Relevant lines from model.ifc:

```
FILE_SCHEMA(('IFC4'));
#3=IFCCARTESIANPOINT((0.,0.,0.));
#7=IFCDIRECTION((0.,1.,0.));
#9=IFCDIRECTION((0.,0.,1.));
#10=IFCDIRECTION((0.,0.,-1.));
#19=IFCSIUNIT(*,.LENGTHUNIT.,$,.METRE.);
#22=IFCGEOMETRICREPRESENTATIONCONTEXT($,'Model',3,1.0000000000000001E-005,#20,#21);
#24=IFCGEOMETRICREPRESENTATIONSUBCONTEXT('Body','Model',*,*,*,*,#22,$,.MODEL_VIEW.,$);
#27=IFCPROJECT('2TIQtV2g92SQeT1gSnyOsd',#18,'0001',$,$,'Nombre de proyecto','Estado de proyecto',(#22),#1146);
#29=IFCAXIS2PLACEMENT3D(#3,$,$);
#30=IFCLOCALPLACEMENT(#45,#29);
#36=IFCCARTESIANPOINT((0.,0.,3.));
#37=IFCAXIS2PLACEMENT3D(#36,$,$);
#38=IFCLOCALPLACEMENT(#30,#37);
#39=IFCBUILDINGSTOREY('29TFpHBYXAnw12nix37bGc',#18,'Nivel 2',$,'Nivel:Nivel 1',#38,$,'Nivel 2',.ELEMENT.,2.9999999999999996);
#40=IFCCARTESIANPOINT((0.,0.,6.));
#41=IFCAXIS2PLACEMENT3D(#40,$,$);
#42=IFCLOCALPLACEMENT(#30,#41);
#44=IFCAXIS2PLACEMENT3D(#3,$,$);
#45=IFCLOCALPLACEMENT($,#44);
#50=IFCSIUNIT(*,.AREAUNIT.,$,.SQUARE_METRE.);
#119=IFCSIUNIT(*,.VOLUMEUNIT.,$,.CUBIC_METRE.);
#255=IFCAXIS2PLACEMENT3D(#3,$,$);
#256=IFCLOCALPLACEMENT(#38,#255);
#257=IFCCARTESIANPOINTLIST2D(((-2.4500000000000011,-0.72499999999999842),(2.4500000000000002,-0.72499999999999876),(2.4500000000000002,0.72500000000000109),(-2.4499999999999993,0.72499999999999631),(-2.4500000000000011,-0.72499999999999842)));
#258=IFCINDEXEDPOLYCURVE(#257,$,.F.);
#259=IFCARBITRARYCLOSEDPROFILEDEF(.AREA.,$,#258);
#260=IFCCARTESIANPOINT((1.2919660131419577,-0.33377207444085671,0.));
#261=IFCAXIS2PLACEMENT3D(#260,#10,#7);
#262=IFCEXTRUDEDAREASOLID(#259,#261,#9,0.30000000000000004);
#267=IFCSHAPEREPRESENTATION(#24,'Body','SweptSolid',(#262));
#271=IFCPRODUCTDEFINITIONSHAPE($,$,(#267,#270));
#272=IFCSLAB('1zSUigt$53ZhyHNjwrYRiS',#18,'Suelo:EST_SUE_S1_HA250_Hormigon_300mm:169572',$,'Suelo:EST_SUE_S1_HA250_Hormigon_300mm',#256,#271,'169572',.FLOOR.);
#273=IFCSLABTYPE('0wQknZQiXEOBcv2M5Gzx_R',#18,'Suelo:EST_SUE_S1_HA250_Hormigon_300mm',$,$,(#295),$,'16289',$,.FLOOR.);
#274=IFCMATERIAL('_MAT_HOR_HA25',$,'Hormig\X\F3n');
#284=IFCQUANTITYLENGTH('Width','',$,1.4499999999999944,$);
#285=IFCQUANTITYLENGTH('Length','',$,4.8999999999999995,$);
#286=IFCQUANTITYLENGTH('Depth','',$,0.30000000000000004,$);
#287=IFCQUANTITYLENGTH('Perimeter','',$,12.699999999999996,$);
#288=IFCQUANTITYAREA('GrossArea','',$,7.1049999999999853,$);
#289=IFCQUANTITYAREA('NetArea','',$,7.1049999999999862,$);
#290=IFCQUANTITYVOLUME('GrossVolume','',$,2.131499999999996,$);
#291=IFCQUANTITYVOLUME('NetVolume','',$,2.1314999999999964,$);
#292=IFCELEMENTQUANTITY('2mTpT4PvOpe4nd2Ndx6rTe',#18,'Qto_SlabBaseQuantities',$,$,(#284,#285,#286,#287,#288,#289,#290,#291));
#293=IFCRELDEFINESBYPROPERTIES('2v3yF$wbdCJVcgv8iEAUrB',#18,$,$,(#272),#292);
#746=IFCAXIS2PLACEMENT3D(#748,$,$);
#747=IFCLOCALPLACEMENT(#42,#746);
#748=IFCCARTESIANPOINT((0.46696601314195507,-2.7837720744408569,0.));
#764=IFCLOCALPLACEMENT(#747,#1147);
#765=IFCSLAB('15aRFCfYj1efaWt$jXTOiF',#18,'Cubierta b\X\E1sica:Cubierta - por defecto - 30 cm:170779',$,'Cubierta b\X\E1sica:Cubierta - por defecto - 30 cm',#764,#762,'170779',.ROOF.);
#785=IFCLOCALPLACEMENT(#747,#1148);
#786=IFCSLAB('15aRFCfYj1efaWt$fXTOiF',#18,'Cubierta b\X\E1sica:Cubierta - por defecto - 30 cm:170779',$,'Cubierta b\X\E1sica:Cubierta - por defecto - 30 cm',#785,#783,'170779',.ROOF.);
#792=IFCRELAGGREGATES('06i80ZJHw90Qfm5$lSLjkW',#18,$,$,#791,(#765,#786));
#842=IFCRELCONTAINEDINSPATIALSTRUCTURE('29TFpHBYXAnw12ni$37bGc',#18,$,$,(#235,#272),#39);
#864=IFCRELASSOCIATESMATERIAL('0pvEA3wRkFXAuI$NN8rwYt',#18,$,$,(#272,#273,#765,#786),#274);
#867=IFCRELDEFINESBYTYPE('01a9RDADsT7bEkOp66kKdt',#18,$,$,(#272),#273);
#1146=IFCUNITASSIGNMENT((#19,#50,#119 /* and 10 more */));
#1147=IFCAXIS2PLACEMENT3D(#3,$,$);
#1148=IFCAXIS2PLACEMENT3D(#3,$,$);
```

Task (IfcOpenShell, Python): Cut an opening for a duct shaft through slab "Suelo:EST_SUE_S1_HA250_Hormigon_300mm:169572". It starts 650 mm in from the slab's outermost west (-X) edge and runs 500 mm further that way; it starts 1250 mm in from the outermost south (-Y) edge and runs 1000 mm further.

```python
import numpy as np
import ifcopenshell
import ifcopenshell.api.feature
import ifcopenshell.api.geometry
import ifcopenshell.api.pset
import ifcopenshell.api.root
import ifcopenshell.geom
import ifcopenshell.util.element
import ifcopenshell.util.placement
import ifcopenshell.util.representation
import ifcopenshell.util.shape
import ifcopenshell.util.unit

model = ifcopenshell.open("model.ifc")
unit_scale = ifcopenshell.util.unit.calculate_unit_scale(model)
area_scale = ifcopenshell.util.unit.calculate_unit_scale(model, "AREAUNIT")
volume_scale = ifcopenshell.util.unit.calculate_unit_scale(model, "VOLUMEUNIT")
settings = ifcopenshell.geom.settings()


def volume(element):
    """Net volume in cubic metres, openings subtracted."""
    shape = ifcopenshell.geom.create_shape(settings, element)
    return ifcopenshell.util.shape.get_volume(shape.geometry)


slab = model.by_guid("1zSUigt$53ZhyHNjwrYRiS")
before = volume(slab)

# Extent in the slab's own axes, in metres. The edges named are its -X and -Y sides.
slab_shape = ifcopenshell.geom.create_shape(settings, slab)
vertices = ifcopenshell.util.shape.get_vertices(slab_shape.geometry)
x_min, y_min, bottom = vertices.min(axis=0)
top = vertices[:, 2].max()

opening = ifcopenshell.api.root.create_entity(model, ifc_class="IfcOpeningElement", name="Duct shaft opening", predefined_type="OPENING")
context = ifcopenshell.util.representation.get_context(model, "Model", "Body", "MODEL_VIEW")
width, depth = 0.5, 1
outline = [(0.0, 0.0), (width, 0.0), (width, depth), (0.0, depth), (0.0, 0.0)]
# Overshoot both faces by 50 mm so the cut is clean.
shape = ifcopenshell.api.geometry.add_slab_representation(
    model, context=context, depth=top - bottom + 0.1, polyline=outline
)
ifcopenshell.api.geometry.assign_representation(model, product=opening, representation=shape)

matrix = ifcopenshell.util.placement.get_local_placement(slab.ObjectPlacement)
matrix[:, 3] = matrix @ np.append(np.array([x_min + 0.65, y_min + 1.25, bottom - 0.05]) / unit_scale, 1.0)
ifcopenshell.api.geometry.edit_object_placement(model, product=opening, matrix=matrix, is_si=False)
ifcopenshell.api.feature.add_feature(model, feature=opening, element=slab)

after = volume(slab)

# Update the slab's stored quantities.
qto = model.by_id(ifcopenshell.util.element.get_pset(slab, "Qto_SlabBaseQuantities", should_inherit=False)["id"])
ifcopenshell.api.pset.edit_qto(model, qto=qto, properties={
    "NetArea": after / (top - bottom) / area_scale,
    "NetVolume": after / volume_scale,
})

print(f"slab volume {before:.3f} -> {after:.3f} m3")

model.write("model_v2.ifc")
```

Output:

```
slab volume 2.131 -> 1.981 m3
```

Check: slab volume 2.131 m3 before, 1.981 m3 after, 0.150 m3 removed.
